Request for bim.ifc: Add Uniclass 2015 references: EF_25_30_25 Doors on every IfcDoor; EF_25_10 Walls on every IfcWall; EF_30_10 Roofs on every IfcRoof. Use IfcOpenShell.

First a look at what the model holds.

```python
import ifcopenshell

model = ifcopenshell.open("bim.ifc")
print(model.schema)
print("classifications:", [c.Name for c in model.by_type("IfcClassification")])
for ifc_class in ("IfcDoor", "IfcRoof", "IfcStair", "IfcWall", "IfcWindow"):
    print(ifc_class, len(model.by_type(ifc_class)))
```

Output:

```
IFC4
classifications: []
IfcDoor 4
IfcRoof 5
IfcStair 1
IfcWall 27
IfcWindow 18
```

```python
import ifcopenshell
import ifcopenshell.api.classification

model = ifcopenshell.open("bim.ifc")

system = ifcopenshell.api.classification.add_classification(model, classification="Uniclass 2015")

codes = {
    "IfcDoor": ("EF_25_30_25", "Doors"),
    "IfcWall": ("EF_25_10", "Walls"),
    "IfcRoof": ("EF_30_10", "Roofs"),
}
for ifc_class, (code, name) in codes.items():
    products = model.by_type(ifc_class)
    ifcopenshell.api.classification.add_reference(
        model, products=products, classification=system, identification=code, name=name
    )
    print(code, len(products))

model.write("bim-out.ifc")
```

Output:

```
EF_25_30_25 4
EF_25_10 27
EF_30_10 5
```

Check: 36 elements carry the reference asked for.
